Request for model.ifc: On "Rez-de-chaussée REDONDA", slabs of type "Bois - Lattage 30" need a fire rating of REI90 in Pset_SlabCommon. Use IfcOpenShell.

First a look at what the model holds.

```python
import ifcopenshell
import ifcopenshell.util.element

model = ifcopenshell.open("model.ifc")
print(model.schema)
storey = next(s for s in model.by_type("IfcBuildingStorey") if s.Name == "Rez-de-chaussée REDONDA")
slabs = [e for e in ifcopenshell.util.element.get_decomposition(storey) if e.is_a("IfcSlab")]
seen = {}
for e in slabs:
    element_type = ifcopenshell.util.element.get_type(e)
    key = (element_type.Name if element_type != e and element_type else None, ifcopenshell.util.element.get_pset(e, "Pset_SlabCommon", "FireRating"))
    seen[key] = seen.get(key, 0) + 1
for (name, value), count in sorted(seen.items(), key=str):
    print(count, "x", name, "|", value)
```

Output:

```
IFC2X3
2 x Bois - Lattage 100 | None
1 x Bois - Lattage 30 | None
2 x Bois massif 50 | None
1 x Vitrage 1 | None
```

```python
import ifcopenshell
import ifcopenshell.api.pset
import ifcopenshell.util.element

model = ifcopenshell.open("model.ifc")

storey = next(s for s in model.by_type("IfcBuildingStorey") if s.Name == "Rez-de-chaussée REDONDA")
slabs = [e for e in ifcopenshell.util.element.get_decomposition(storey) if e.is_a("IfcSlab")]

count = 0
for e in slabs:
    element_type = ifcopenshell.util.element.get_type(e)
    if element_type in (None, e) or element_type.Name != "Bois - Lattage 30":
        continue
    # add_pset returns the element's existing set when there is one.
    pset = ifcopenshell.api.pset.add_pset(model, product=e, name="Pset_SlabCommon")
    ifcopenshell.api.pset.edit_pset(model, pset=pset, properties={"FireRating": "REI90"})
    count += 1

print(count, "slabs updated")

model.write("model_updated.ifc")
```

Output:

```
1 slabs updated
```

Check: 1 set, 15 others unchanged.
